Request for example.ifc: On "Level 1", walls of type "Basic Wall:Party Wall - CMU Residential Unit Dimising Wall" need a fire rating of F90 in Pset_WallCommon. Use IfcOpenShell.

First a look at what the model holds.

```python
import ifcopenshell
import ifcopenshell.util.element

model = ifcopenshell.open("example.ifc")
print(model.schema)
storey = next(s for s in model.by_type("IfcBuildingStorey") if s.Name == "Level 1")
walls = [e for e in ifcopenshell.util.element.get_decomposition(storey) if e.is_a("IfcWall")]
seen = {}
for e in walls:
    element_type = ifcopenshell.util.element.get_type(e)
    key = (element_type.Name if element_type != e and element_type else None, ifcopenshell.util.element.get_pset(e, "Pset_WallCommon", "FireRating"))
    seen[key] = seen.get(key, 0) + 1
for (name, value), count in sorted(seen.items(), key=str):
    print(count, "x", name, "|", value)
```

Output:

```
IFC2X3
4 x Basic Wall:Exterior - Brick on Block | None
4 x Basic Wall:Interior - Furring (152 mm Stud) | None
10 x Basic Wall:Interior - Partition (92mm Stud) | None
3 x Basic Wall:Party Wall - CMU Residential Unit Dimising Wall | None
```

```python
import ifcopenshell
import ifcopenshell.api.pset
import ifcopenshell.util.element

model = ifcopenshell.open("example.ifc")

storey = next(s for s in model.by_type("IfcBuildingStorey") if s.Name == "Level 1")
walls = [e for e in ifcopenshell.util.element.get_decomposition(storey) if e.is_a("IfcWall")]

count = 0
for e in walls:
    element_type = ifcopenshell.util.element.get_type(e)
    if element_type in (None, e) or element_type.Name != "Basic Wall:Party Wall - CMU Residential Unit Dimising Wall":
        continue
    # add_pset returns the element's existing set when there is one.
    pset = ifcopenshell.api.pset.add_pset(model, product=e, name="Pset_WallCommon")
    ifcopenshell.api.pset.edit_pset(model, pset=pset, properties={"FireRating": "F90"})
    count += 1

print(count, "walls updated")

model.write("example_edited.ifc")
```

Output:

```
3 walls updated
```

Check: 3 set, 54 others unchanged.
